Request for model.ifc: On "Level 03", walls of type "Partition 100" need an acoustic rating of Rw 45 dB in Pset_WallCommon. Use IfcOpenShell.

First a look at what the model holds.

```python
import ifcopenshell
import ifcopenshell.util.element

model = ifcopenshell.open("model.ifc")
print(model.schema)
storey = next(s for s in model.by_type("IfcBuildingStorey") if s.Name == "Level 03")
walls = [e for e in ifcopenshell.util.element.get_decomposition(storey) if e.is_a("IfcWall")]
seen = {}
for e in walls:
    element_type = ifcopenshell.util.element.get_type(e)
    key = (element_type.Name if element_type != e and element_type else None, ifcopenshell.util.element.get_pset(e, "Pset_WallCommon", "AcousticRating"))
    seen[key] = seen.get(key, 0) + 1
for (name, value), count in sorted(seen.items(), key=str):
    print(count, "x", name, "|", value)
```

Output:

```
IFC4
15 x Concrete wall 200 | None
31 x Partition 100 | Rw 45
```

```python
import ifcopenshell
import ifcopenshell.api.pset
import ifcopenshell.util.element

model = ifcopenshell.open("model.ifc")

storey = next(s for s in model.by_type("IfcBuildingStorey") if s.Name == "Level 03")
walls = [e for e in ifcopenshell.util.element.get_decomposition(storey) if e.is_a("IfcWall")]

count = 0
for e in walls:
    element_type = ifcopenshell.util.element.get_type(e)
    if element_type in (None, e) or element_type.Name != "Partition 100":
        continue
    # add_pset returns the element's existing set when there is one.
    pset = ifcopenshell.api.pset.add_pset(model, product=e, name="Pset_WallCommon")
    ifcopenshell.api.pset.edit_pset(model, pset=pset, properties={"AcousticRating": "Rw 45 dB"})
    count += 1

print(count, "walls updated")

model.write("model_rev.ifc")
```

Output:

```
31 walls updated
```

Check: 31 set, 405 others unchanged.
